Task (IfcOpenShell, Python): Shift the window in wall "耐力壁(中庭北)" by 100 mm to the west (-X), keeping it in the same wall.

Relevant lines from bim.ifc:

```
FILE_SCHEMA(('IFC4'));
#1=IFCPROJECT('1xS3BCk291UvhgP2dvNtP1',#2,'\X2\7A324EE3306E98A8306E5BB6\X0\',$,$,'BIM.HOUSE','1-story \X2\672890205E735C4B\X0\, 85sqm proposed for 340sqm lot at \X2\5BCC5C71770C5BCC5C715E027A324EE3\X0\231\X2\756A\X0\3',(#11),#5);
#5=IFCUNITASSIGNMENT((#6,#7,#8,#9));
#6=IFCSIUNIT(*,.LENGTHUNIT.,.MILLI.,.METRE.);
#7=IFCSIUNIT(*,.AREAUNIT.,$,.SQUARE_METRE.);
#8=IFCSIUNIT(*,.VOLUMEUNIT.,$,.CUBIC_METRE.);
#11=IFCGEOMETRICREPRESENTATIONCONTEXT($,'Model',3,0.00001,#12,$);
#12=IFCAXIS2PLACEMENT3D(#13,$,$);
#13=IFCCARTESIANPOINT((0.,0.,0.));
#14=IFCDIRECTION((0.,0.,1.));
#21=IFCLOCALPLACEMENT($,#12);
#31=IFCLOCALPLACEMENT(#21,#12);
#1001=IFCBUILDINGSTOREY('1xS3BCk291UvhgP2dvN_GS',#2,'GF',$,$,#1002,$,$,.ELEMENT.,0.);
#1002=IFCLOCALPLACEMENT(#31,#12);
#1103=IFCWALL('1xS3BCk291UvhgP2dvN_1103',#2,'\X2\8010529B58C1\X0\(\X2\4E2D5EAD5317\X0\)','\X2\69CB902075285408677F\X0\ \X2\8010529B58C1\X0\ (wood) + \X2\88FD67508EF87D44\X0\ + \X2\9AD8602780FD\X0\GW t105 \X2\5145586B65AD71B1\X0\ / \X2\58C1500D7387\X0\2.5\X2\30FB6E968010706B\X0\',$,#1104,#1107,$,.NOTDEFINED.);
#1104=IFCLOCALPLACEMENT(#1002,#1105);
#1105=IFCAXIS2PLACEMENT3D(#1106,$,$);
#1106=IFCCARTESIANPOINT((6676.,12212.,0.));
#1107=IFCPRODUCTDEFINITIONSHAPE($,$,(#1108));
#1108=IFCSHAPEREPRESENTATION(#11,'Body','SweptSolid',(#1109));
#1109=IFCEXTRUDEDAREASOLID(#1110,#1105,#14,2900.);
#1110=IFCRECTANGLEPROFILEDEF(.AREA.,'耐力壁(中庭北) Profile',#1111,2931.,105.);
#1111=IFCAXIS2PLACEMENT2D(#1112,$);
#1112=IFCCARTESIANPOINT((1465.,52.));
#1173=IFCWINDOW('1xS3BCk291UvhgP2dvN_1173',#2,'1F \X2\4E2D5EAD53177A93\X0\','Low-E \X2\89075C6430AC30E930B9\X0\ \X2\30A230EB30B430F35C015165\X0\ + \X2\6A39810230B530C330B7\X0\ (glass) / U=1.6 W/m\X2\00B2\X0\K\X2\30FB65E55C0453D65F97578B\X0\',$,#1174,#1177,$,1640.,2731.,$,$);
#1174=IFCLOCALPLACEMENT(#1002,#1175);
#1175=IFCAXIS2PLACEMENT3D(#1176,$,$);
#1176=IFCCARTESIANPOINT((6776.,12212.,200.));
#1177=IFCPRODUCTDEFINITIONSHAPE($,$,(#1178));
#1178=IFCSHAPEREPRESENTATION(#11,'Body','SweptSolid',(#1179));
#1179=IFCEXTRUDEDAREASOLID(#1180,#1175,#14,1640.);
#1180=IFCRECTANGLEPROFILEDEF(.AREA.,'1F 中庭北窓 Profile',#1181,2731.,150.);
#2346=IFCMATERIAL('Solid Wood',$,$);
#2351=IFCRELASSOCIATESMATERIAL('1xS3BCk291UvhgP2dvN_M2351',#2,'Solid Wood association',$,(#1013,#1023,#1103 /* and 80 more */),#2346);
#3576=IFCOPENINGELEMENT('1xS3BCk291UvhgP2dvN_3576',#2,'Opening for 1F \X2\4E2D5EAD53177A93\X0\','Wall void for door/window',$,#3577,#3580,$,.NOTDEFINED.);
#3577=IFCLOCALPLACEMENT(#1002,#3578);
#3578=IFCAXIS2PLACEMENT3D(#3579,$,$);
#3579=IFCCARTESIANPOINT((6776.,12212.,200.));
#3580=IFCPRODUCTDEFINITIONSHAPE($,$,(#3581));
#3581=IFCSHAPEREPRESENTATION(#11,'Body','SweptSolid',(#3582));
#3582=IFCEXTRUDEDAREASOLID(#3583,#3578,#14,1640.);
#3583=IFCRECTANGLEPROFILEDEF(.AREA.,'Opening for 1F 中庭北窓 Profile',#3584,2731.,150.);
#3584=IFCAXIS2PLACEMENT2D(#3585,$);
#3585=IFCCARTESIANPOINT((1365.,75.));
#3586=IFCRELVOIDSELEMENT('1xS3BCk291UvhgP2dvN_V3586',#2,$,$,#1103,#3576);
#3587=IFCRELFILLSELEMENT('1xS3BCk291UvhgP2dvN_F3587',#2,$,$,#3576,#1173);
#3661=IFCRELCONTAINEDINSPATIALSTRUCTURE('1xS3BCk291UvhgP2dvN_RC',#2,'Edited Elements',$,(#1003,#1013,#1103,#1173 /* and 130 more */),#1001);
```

```python
import ifcopenshell
import ifcopenshell.api.geometry
import ifcopenshell.util.placement
import ifcopenshell.util.unit

model = ifcopenshell.open("bim.ifc")
unit_scale = ifcopenshell.util.unit.calculate_unit_scale(model)

window = model.by_id(1173)
opening = window.FillsVoids[0].RelatingOpeningElement
wall = opening.VoidsElements[0].RelatingBuildingElement

wall_matrix = ifcopenshell.util.placement.get_local_placement(wall.ObjectPlacement)
shift = wall_matrix[:3, 0] * -0.1 / unit_scale
before = ifcopenshell.util.placement.get_local_placement(window.ObjectPlacement)[:3, 3].copy()

# The window is not placed relative to its opening, so move both.
for product in (opening, window):
    matrix = ifcopenshell.util.placement.get_local_placement(product.ObjectPlacement)
    matrix[:3, 3] += shift
    ifcopenshell.api.geometry.edit_object_placement(model, product=product, matrix=matrix, is_si=False)

after = ifcopenshell.util.placement.get_local_placement(window.ObjectPlacement)[:3, 3]
print("window moved by", (after - before).round(3) + 0.0)

model.write("bim_v2.ifc")
```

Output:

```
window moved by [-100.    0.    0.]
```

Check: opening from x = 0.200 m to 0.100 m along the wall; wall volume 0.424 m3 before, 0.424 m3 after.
